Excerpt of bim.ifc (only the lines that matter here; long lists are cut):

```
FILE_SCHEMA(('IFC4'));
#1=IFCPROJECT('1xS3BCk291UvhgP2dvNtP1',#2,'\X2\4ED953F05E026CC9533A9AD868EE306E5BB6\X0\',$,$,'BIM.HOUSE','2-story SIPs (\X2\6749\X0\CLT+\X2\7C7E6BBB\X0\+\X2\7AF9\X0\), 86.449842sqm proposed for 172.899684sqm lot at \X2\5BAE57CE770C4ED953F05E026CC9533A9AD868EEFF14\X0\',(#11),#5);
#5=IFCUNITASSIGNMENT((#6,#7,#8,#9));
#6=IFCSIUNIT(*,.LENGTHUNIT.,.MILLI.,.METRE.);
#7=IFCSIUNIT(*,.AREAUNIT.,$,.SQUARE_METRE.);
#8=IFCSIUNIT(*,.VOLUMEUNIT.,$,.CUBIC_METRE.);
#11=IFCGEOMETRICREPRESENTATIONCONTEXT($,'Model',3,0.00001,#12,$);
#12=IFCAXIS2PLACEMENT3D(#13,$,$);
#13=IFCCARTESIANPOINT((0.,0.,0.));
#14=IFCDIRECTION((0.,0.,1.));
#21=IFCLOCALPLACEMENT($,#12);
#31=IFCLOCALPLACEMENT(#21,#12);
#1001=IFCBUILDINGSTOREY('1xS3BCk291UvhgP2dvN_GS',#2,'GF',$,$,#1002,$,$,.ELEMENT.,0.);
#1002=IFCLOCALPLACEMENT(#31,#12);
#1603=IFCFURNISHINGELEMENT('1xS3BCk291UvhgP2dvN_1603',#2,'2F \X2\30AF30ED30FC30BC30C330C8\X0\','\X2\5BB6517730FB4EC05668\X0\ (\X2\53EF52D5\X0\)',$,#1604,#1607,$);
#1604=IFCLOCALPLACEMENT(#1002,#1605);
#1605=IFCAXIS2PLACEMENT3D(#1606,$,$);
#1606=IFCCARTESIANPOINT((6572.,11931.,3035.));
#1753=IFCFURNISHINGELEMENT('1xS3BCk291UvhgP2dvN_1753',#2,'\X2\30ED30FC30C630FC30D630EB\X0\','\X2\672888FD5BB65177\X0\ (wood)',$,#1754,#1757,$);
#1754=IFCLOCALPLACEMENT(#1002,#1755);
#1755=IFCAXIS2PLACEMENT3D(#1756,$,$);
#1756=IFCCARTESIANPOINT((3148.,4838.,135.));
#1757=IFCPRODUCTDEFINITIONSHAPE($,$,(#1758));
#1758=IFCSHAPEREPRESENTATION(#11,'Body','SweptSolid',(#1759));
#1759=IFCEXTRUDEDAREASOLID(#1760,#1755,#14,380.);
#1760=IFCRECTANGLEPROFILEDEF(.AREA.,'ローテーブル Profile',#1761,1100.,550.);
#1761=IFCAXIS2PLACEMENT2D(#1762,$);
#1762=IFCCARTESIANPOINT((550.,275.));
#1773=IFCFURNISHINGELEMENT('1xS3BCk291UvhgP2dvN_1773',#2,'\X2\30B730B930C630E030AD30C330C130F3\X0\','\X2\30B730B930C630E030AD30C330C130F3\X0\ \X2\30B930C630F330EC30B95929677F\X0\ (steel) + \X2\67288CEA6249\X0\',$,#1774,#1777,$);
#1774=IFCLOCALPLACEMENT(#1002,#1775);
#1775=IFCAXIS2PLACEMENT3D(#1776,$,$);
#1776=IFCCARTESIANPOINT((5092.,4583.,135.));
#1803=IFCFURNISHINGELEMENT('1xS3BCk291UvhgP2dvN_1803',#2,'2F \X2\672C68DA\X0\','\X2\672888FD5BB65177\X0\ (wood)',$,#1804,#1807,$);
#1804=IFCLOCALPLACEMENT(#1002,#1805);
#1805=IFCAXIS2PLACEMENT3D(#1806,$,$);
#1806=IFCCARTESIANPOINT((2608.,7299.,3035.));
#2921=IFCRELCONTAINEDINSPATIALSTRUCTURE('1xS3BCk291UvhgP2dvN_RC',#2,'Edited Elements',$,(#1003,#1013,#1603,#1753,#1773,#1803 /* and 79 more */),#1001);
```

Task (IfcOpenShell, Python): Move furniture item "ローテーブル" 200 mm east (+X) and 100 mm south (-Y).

```python
import ifcopenshell
import ifcopenshell.api.geometry
import ifcopenshell.util.placement
import ifcopenshell.util.unit

model = ifcopenshell.open("bim.ifc")
unit_scale = ifcopenshell.util.unit.calculate_unit_scale(model)

item = model.by_id(1753)
matrix = ifcopenshell.util.placement.get_local_placement(item.ObjectPlacement)
matrix[0, 3] += 0.2 / unit_scale
matrix[1, 3] -= 0.1 / unit_scale
ifcopenshell.api.geometry.edit_object_placement(model, product=item, matrix=matrix, is_si=False)

print(ifcopenshell.util.placement.get_local_placement(item.ObjectPlacement).round(3) + 0.0)

model.write("bim_edited.ifc")
```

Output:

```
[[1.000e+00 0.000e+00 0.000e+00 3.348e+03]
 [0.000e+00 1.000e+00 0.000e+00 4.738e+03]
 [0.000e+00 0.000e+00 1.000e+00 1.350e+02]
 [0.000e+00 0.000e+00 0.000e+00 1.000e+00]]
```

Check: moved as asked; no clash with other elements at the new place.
